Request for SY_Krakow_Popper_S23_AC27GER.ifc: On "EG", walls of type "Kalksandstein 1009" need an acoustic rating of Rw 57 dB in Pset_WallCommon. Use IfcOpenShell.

First a look at what the model holds.

```python
import ifcopenshell
import ifcopenshell.util.element

model = ifcopenshell.open("SY_Krakow_Popper_S23_AC27GER.ifc")
print(model.schema)
storey = next(s for s in model.by_type("IfcBuildingStorey") if s.Name == "EG")
walls = [e for e in ifcopenshell.util.element.get_decomposition(storey) if e.is_a("IfcWall")]
seen = {}
for e in walls:
    element_type = ifcopenshell.util.element.get_type(e)
    key = (element_type.Name if element_type != e and element_type else None, ifcopenshell.util.element.get_pset(e, "Pset_WallCommon", "AcousticRating"))
    seen[key] = seen.get(key, 0) + 1
for (name, value), count in sorted(seen.items(), key=str):
    print(count, "x", name, "|", value)
```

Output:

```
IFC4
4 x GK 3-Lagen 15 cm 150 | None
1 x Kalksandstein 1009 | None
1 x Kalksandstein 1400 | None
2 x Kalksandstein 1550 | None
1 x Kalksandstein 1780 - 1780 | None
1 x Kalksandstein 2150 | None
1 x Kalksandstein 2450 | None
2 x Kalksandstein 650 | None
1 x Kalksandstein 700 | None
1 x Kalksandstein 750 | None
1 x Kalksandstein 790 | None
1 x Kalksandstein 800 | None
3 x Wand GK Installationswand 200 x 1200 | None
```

```python
import ifcopenshell
import ifcopenshell.api.pset
import ifcopenshell.util.element

model = ifcopenshell.open("SY_Krakow_Popper_S23_AC27GER.ifc")

storey = next(s for s in model.by_type("IfcBuildingStorey") if s.Name == "EG")
walls = [e for e in ifcopenshell.util.element.get_decomposition(storey) if e.is_a("IfcWall")]

count = 0
for e in walls:
    element_type = ifcopenshell.util.element.get_type(e)
    if element_type in (None, e) or element_type.Name != "Kalksandstein 1009":
        continue
    # add_pset returns the element's existing set when there is one.
    pset = ifcopenshell.api.pset.add_pset(model, product=e, name="Pset_WallCommon")
    ifcopenshell.api.pset.edit_pset(model, pset=pset, properties={"AcousticRating": "Rw 57 dB"})
    count += 1

print(count, "walls updated")

model.write("SY_Krakow_Popper_S23_AC27GER_updated.ifc")
```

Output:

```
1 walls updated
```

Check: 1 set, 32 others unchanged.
